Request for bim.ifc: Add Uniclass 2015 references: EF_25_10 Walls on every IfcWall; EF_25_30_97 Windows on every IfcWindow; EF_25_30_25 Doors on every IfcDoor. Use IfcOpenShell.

First a look at what the model holds.

```python
import ifcopenshell

model = ifcopenshell.open("bim.ifc")
print(model.schema)
print("classifications:", [c.Name for c in model.by_type("IfcClassification")])
for ifc_class in ("IfcDoor", "IfcRoof", "IfcStair", "IfcWall", "IfcWindow"):
    print(ifc_class, len(model.by_type(ifc_class)))
```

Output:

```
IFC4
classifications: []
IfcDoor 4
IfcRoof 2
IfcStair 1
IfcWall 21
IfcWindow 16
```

```python
import ifcopenshell
import ifcopenshell.api.classification

model = ifcopenshell.open("bim.ifc")

system = ifcopenshell.api.classification.add_classification(model, classification="Uniclass 2015")

codes = {
    "IfcWall": ("EF_25_10", "Walls"),
    "IfcWindow": ("EF_25_30_97", "Windows"),
    "IfcDoor": ("EF_25_30_25", "Doors"),
}
for ifc_class, (code, name) in codes.items():
    products = model.by_type(ifc_class)
    ifcopenshell.api.classification.add_reference(
        model, products=products, classification=system, identification=code, name=name
    )
    print(code, len(products))

model.write("bim_rev.ifc")
```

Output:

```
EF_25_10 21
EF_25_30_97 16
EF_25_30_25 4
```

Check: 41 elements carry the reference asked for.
